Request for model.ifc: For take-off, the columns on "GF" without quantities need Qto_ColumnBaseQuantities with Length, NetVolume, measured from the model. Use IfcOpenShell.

First a look at what the model holds.

```python
import ifcopenshell
import ifcopenshell.util.element
import ifcopenshell.util.unit

model = ifcopenshell.open("model.ifc")
print(model.schema)
for unit_type in ("LENGTHUNIT", "AREAUNIT", "VOLUMEUNIT"):
    print(unit_type, ifcopenshell.util.unit.calculate_unit_scale(model, unit_type))
storey = next(s for s in model.by_type("IfcBuildingStorey") if s.Name == "GF")
columns = [e for e in ifcopenshell.util.element.get_decomposition(storey) if e.is_a("IfcColumn")]
for e in sorted(columns, key=lambda e: e.id()):
    print(e.id(), e.is_a(), e.Name, list(ifcopenshell.util.element.get_psets(e, qtos_only=True)), sep=" | ")
```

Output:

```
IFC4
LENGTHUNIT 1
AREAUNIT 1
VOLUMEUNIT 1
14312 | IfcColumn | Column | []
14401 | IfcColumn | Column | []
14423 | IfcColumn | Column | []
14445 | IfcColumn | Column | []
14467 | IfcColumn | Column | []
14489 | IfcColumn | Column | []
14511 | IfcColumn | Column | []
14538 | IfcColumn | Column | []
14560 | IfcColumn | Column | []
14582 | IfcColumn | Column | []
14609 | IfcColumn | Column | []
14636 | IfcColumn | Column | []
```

```python
import ifcopenshell
import ifcopenshell.api.pset
import ifcopenshell.geom
import ifcopenshell.util.element
import ifcopenshell.util.shape
import ifcopenshell.util.unit

model = ifcopenshell.open("model.ifc")
unit_scale = ifcopenshell.util.unit.calculate_unit_scale(model)
volume_scale = ifcopenshell.util.unit.calculate_unit_scale(model, "VOLUMEUNIT")
settings = ifcopenshell.geom.settings()

storey = next(s for s in model.by_type("IfcBuildingStorey") if s.Name == "GF")
columns = [e for e in ifcopenshell.util.element.get_decomposition(storey) if e.is_a("IfcColumn")]

for e in sorted(columns, key=lambda e: e.id()):
    if ifcopenshell.util.element.get_psets(e, qtos_only=True, should_inherit=False):
        continue
    # Geometry comes back in metres, in the element's own axes.
    shape = ifcopenshell.geom.create_shape(settings, e)
    values = {
        "Length": ifcopenshell.util.shape.get_z(shape.geometry) / unit_scale,
        "NetVolume": ifcopenshell.util.shape.get_volume(shape.geometry) / volume_scale,
    }
    qto = ifcopenshell.api.pset.add_qto(model, product=e, name="Qto_ColumnBaseQuantities")
    ifcopenshell.api.pset.edit_qto(model, qto=qto, properties=values)
    print(e.id(), {k: round(v, 3) for k, v in values.items()})

model.write("model_updated.ifc")
```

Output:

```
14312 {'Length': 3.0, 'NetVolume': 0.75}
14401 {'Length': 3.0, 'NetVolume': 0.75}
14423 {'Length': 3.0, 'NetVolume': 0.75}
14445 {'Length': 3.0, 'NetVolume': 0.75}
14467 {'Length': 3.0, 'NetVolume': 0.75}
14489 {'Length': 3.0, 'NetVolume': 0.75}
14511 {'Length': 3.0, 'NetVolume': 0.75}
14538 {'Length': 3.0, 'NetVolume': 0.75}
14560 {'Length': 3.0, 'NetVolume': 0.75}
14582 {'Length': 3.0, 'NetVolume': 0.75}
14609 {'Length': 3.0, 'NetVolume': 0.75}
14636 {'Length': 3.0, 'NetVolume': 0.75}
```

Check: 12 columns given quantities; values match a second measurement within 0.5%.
